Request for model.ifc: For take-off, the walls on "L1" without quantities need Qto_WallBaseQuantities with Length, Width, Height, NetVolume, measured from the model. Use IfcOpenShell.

First a look at what the model holds.

```python
import ifcopenshell
import ifcopenshell.util.element
import ifcopenshell.util.unit

model = ifcopenshell.open("model.ifc")
print(model.schema)
for unit_type in ("LENGTHUNIT", "AREAUNIT", "VOLUMEUNIT"):
    print(unit_type, ifcopenshell.util.unit.calculate_unit_scale(model, unit_type))
storey = next(s for s in model.by_type("IfcBuildingStorey") if s.Name == "L1")
walls = [e for e in ifcopenshell.util.element.get_decomposition(storey) if e.is_a("IfcWall")]
for e in sorted(walls, key=lambda e: e.id()):
    print(e.id(), e.is_a(), e.Name, list(ifcopenshell.util.element.get_psets(e, qtos_only=True)), sep=" | ")
```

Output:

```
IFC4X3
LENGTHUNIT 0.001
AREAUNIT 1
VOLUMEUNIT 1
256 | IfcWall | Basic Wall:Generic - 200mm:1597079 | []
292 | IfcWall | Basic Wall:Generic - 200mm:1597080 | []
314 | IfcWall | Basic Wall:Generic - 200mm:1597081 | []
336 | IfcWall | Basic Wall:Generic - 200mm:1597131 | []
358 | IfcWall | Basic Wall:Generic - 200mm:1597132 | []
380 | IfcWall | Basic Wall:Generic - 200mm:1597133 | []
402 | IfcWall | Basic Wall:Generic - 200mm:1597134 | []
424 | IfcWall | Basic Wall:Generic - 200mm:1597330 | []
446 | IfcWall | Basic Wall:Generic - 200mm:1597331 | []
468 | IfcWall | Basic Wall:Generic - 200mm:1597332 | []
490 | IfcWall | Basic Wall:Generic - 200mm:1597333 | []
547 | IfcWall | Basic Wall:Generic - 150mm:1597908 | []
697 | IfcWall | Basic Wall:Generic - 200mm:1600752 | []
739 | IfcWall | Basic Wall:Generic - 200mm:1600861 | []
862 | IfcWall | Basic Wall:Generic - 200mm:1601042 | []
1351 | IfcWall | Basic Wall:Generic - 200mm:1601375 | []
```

```python
import ifcopenshell
import ifcopenshell.api.pset
import ifcopenshell.geom
import ifcopenshell.util.element
import ifcopenshell.util.shape
import ifcopenshell.util.unit

model = ifcopenshell.open("model.ifc")
unit_scale = ifcopenshell.util.unit.calculate_unit_scale(model)
volume_scale = ifcopenshell.util.unit.calculate_unit_scale(model, "VOLUMEUNIT")
settings = ifcopenshell.geom.settings()

storey = next(s for s in model.by_type("IfcBuildingStorey") if s.Name == "L1")
walls = [e for e in ifcopenshell.util.element.get_decomposition(storey) if e.is_a("IfcWall")]

for e in sorted(walls, key=lambda e: e.id()):
    if ifcopenshell.util.element.get_psets(e, qtos_only=True, should_inherit=False):
        continue
    # Geometry comes back in metres, in the element's own axes.
    shape = ifcopenshell.geom.create_shape(settings, e)
    values = {
        "Length": ifcopenshell.util.shape.get_x(shape.geometry) / unit_scale,
        "Width": ifcopenshell.util.shape.get_y(shape.geometry) / unit_scale,
        "Height": ifcopenshell.util.shape.get_z(shape.geometry) / unit_scale,
        "NetVolume": ifcopenshell.util.shape.get_volume(shape.geometry) / volume_scale,
    }
    qto = ifcopenshell.api.pset.add_qto(model, product=e, name="Qto_WallBaseQuantities")
    ifcopenshell.api.pset.edit_qto(model, qto=qto, properties=values)
    print(e.id(), {k: round(v, 3) for k, v in values.items()})

model.write("model_updated.ifc")
```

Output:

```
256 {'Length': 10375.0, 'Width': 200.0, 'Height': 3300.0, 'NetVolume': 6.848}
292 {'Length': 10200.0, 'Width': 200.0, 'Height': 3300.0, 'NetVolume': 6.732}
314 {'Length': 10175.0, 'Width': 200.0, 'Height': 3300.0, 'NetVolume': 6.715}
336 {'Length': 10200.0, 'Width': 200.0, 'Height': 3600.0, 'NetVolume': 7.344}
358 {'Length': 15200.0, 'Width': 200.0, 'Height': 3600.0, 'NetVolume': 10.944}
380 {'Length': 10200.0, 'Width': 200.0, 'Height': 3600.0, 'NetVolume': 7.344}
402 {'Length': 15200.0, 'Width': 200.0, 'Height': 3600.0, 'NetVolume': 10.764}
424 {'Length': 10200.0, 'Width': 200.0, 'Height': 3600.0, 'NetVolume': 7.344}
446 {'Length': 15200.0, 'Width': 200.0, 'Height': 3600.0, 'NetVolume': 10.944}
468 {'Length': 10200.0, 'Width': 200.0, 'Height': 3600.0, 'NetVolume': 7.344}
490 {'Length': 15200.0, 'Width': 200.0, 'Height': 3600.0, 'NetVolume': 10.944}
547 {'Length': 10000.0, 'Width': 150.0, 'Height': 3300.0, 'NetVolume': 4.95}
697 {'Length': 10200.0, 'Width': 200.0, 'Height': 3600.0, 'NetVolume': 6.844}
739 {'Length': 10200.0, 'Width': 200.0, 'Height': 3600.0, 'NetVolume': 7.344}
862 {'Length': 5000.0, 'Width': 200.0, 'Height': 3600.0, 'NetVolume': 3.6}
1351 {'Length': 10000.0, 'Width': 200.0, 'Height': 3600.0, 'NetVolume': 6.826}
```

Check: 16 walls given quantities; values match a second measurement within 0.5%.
